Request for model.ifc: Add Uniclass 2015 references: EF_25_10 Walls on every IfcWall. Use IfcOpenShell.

First a look at what the model holds.

```python
import ifcopenshell

model = ifcopenshell.open("model.ifc")
print(model.schema)
print("classifications:", [c.Name for c in model.by_type("IfcClassification")])
for ifc_class in ("IfcDoor", "IfcRoof", "IfcStair", "IfcWall", "IfcWindow"):
    print(ifc_class, len(model.by_type(ifc_class)))
```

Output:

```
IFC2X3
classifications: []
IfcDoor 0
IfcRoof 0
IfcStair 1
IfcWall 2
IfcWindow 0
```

```python
import ifcopenshell
import ifcopenshell.api.classification

model = ifcopenshell.open("model.ifc")

# IFC2X3 requires Source and Edition and has no link from the project to the system.
system = model.create_entity("IfcClassification", Source="NBS", Edition="2015", Name="Uniclass 2015")

codes = {
    "IfcWall": ("EF_25_10", "Walls"),
}
for ifc_class, (code, name) in codes.items():
    products = model.by_type(ifc_class)
    ifcopenshell.api.classification.add_reference(
        model, products=products, classification=system, identification=code, name=name
    )
    print(code, len(products))

model.write("model_v2.ifc")
```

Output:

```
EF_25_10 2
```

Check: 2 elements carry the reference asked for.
